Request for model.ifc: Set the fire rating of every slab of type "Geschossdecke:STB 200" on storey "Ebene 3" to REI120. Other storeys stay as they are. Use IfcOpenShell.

First a look at what the model holds.

```python
import ifcopenshell
import ifcopenshell.util.element

model = ifcopenshell.open("model.ifc")
print(model.schema)
storey = next(s for s in model.by_type("IfcBuildingStorey") if s.Name == "Ebene 3")
slabs = [e for e in ifcopenshell.util.element.get_decomposition(storey) if e.is_a("IfcSlab")]
seen = {}
for e in slabs:
    element_type = ifcopenshell.util.element.get_type(e)
    key = (element_type.Name if element_type != e and element_type else None, ifcopenshell.util.element.get_pset(e, "Pset_SlabCommon", "FireRating"))
    seen[key] = seen.get(key, 0) + 1
for (name, value), count in sorted(seen.items(), key=str):
    print(count, "x", name, "|", value)
```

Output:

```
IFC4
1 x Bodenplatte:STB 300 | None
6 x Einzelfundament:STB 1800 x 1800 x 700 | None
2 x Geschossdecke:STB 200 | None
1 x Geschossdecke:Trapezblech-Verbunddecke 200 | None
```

```python
import ifcopenshell
import ifcopenshell.api.pset
import ifcopenshell.util.element

model = ifcopenshell.open("model.ifc")

storey = next(s for s in model.by_type("IfcBuildingStorey") if s.Name == "Ebene 3")
slabs = [e for e in ifcopenshell.util.element.get_decomposition(storey) if e.is_a("IfcSlab")]

count = 0
for e in slabs:
    element_type = ifcopenshell.util.element.get_type(e)
    if element_type in (None, e) or element_type.Name != "Geschossdecke:STB 200":
        continue
    # add_pset returns the element's existing set when there is one.
    pset = ifcopenshell.api.pset.add_pset(model, product=e, name="Pset_SlabCommon")
    ifcopenshell.api.pset.edit_pset(model, pset=pset, properties={"FireRating": "REI120"})
    count += 1

print(count, "slabs updated")

model.write("model_v2.ifc")
```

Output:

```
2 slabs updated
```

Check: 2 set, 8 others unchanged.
